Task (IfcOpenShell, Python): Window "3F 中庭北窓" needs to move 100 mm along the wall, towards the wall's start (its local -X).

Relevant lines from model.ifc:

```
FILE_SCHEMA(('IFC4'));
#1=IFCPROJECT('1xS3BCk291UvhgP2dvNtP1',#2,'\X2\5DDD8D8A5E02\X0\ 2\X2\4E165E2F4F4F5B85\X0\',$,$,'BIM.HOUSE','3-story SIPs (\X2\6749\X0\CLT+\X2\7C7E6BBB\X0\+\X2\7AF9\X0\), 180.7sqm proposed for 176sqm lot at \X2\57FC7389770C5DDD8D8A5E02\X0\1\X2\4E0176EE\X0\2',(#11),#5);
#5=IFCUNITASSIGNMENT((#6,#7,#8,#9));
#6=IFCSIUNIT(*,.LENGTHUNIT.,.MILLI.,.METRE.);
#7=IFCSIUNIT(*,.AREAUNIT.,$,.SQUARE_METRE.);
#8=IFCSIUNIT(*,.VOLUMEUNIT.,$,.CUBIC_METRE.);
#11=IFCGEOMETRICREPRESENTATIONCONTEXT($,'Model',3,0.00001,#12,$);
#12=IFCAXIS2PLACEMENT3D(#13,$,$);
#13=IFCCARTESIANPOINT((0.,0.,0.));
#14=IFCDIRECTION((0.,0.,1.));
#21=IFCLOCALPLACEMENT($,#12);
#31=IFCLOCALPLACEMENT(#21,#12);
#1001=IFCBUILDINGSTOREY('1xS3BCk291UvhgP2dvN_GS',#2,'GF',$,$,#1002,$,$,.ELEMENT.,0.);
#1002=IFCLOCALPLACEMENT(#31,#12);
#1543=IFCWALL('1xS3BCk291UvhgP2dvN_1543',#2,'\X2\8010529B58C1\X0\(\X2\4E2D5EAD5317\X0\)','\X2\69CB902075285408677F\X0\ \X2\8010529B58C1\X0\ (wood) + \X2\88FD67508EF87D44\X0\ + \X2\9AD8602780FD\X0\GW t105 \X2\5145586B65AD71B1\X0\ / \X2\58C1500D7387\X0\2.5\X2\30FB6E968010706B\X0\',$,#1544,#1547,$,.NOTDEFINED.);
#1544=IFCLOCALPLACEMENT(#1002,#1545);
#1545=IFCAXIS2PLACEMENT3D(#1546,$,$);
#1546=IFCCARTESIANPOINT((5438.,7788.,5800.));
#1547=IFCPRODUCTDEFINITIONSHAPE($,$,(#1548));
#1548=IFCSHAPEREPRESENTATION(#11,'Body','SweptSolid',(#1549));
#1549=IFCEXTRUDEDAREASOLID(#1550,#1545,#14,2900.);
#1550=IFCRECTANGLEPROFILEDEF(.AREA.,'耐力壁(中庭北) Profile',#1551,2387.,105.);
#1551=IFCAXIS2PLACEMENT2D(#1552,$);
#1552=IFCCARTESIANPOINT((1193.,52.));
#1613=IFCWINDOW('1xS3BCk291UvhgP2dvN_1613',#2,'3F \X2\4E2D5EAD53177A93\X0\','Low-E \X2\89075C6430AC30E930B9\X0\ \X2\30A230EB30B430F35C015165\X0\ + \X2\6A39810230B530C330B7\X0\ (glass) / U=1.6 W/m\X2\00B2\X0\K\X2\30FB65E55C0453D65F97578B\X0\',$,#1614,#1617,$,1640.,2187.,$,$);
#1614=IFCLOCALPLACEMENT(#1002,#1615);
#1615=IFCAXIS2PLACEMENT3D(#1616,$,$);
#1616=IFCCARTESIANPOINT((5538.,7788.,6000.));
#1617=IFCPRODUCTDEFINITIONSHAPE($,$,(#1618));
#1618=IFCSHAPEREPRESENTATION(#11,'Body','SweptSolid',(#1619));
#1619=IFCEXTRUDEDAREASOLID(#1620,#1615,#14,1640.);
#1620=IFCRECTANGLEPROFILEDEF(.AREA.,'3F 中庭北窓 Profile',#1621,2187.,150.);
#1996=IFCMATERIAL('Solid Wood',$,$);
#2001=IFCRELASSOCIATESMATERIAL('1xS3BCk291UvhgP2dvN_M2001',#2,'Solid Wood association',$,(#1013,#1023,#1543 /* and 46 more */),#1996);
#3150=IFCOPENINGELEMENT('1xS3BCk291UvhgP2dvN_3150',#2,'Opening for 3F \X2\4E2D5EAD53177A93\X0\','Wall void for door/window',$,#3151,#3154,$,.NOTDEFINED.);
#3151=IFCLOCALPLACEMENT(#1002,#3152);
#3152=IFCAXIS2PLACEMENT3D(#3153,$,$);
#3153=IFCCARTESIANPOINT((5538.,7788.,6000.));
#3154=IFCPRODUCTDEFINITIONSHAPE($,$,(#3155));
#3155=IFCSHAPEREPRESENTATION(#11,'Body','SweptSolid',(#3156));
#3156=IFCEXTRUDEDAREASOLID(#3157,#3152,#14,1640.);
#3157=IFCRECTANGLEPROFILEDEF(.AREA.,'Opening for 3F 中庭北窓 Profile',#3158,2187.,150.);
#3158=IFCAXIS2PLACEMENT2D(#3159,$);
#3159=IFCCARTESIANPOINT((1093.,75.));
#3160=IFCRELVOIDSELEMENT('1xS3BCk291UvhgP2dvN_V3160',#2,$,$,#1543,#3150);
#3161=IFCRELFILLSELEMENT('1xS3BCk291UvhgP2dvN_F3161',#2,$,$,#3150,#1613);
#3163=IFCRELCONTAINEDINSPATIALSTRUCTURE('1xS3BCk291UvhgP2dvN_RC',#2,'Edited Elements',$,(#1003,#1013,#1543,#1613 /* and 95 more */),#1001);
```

```python
import ifcopenshell
import ifcopenshell.api.geometry
import ifcopenshell.util.placement
import ifcopenshell.util.unit

model = ifcopenshell.open("model.ifc")
unit_scale = ifcopenshell.util.unit.calculate_unit_scale(model)

window = model.by_guid("1xS3BCk291UvhgP2dvN_1613")
opening = window.FillsVoids[0].RelatingOpeningElement
wall = opening.VoidsElements[0].RelatingBuildingElement

wall_matrix = ifcopenshell.util.placement.get_local_placement(wall.ObjectPlacement)
shift = wall_matrix[:3, 0] * -0.1 / unit_scale
before = ifcopenshell.util.placement.get_local_placement(window.ObjectPlacement)[:3, 3].copy()

# The window is not placed relative to its opening, so move both.
for product in (opening, window):
    matrix = ifcopenshell.util.placement.get_local_placement(product.ObjectPlacement)
    matrix[:3, 3] += shift
    ifcopenshell.api.geometry.edit_object_placement(model, product=product, matrix=matrix, is_si=False)

after = ifcopenshell.util.placement.get_local_placement(window.ObjectPlacement)[:3, 3]
print("window moved by", (after - before).round(3) + 0.0)

model.write("model_rev.ifc")
```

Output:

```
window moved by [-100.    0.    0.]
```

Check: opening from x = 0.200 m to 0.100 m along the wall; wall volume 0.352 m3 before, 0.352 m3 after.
